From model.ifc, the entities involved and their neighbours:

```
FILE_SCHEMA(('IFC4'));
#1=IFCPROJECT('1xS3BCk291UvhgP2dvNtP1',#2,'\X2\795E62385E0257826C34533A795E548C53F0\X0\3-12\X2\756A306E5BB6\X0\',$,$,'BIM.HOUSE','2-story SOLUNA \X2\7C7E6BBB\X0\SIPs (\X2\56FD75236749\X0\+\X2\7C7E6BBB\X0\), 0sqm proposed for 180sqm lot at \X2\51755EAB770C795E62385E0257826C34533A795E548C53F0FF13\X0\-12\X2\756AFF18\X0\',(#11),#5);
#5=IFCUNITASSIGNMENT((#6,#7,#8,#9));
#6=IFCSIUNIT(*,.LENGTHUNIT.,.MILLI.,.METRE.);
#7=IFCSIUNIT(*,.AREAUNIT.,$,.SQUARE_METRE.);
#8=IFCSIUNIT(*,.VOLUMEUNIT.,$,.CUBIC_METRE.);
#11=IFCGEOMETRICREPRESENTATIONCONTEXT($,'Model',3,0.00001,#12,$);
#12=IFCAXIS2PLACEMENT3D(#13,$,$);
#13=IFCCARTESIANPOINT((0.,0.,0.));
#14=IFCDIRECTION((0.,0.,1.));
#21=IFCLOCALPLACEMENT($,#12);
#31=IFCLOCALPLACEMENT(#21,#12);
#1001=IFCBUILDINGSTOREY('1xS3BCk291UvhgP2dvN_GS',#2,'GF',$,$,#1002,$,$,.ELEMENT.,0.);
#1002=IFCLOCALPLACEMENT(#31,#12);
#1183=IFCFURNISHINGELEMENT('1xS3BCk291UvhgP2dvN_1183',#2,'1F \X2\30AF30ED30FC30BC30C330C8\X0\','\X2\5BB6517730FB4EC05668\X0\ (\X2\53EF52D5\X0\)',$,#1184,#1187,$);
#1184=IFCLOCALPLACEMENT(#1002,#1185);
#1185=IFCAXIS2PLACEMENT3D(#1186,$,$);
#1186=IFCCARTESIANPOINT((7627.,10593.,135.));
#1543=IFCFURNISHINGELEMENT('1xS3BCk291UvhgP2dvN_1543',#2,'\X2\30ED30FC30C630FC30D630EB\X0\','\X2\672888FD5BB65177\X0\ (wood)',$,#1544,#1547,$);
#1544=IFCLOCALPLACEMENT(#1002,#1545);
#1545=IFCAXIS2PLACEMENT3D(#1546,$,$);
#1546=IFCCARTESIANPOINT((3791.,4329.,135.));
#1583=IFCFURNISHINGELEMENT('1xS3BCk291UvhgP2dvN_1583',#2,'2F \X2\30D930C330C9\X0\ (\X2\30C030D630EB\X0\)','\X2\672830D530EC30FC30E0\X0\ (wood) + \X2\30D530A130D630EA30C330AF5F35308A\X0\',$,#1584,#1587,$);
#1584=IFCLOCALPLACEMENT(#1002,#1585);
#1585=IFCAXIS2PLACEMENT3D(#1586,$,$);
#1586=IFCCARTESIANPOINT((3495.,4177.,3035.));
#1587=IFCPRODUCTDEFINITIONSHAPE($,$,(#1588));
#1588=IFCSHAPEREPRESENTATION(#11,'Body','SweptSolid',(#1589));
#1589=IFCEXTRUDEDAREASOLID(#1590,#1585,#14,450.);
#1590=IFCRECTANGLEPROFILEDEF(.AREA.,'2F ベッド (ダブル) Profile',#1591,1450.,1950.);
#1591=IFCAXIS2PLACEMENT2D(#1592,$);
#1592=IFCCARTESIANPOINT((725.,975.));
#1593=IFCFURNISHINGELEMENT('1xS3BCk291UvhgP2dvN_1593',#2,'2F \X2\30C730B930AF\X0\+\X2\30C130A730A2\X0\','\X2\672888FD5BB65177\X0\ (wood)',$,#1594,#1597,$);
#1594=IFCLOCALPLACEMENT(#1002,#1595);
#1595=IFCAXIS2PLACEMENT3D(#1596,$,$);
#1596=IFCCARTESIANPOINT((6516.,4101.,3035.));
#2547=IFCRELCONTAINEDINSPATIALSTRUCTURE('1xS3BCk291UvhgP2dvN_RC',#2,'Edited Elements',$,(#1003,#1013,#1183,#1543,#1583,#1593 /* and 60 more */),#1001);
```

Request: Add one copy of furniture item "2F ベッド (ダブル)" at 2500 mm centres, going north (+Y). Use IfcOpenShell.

```python
import numpy as np
import ifcopenshell
import ifcopenshell.api.geometry
import ifcopenshell.api.root
import ifcopenshell.util.element
import ifcopenshell.util.placement

model = ifcopenshell.open("model.ifc")


def reuse_history(source, copy):
    """copy_class also copies each property set's owner history, people and application; keep the originals."""
    for rel in copy.IsDefinedBy:
        if rel.is_a("IfcRelDefinesByProperties") and (history := rel.RelatingPropertyDefinition.OwnerHistory):
            rel.RelatingPropertyDefinition.OwnerHistory = source.OwnerHistory
            ifcopenshell.util.element.remove_deep2(model, history)


source = model.by_guid("1xS3BCk291UvhgP2dvN_1583")
base = ifcopenshell.util.placement.get_local_placement(source.ObjectPlacement)
step = np.array([0.0, 1.0, 0.0]) * 2500.0

for i in range(1, 2):
    copy = ifcopenshell.api.root.copy_class(model, product=source)
    copy.Representation = ifcopenshell.util.element.copy_deep(
        model, source.Representation, exclude=["IfcGeometricRepresentationContext", "IfcRepresentationMap"]
    )
    reuse_history(source, copy)
    matrix = base.copy()
    matrix[:3, 3] += i * step
    print("added at", matrix[:3, 3].round(3) + 0.0)
    ifcopenshell.api.geometry.edit_object_placement(model, product=copy, matrix=matrix, is_si=False)

model.write("model_v2.ifc")
```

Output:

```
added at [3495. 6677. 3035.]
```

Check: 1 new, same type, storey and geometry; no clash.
